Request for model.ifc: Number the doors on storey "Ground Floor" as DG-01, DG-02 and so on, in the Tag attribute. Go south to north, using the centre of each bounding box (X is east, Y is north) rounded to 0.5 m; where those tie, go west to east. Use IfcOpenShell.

First a look at what the model holds.

```python
import ifcopenshell
import ifcopenshell.util.element
import ifcopenshell.util.placement

model = ifcopenshell.open("model.ifc")
print(model.schema)
storey = next(s for s in model.by_type("IfcBuildingStorey") if s.Name == "Ground Floor")
doors = [e for e in ifcopenshell.util.element.get_decomposition(storey) if e.is_a("IfcDoor")]
for e in sorted(doors, key=lambda e: e.id()):
    origin = ifcopenshell.util.placement.get_local_placement(e.ObjectPlacement)[:3, 3]
    print(e.id(), e.Tag, e.Name, origin.round(2) + 0.0, sep=" | ")
```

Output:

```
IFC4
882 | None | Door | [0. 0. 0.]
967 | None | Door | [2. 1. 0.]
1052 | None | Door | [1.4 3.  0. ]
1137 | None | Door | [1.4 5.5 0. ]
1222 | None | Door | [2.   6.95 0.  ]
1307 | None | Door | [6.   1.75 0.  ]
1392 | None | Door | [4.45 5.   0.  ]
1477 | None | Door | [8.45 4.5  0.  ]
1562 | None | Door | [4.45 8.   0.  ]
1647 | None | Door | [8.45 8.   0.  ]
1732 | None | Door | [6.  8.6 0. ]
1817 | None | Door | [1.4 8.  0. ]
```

```python
import ifcopenshell
import ifcopenshell.geom
import ifcopenshell.util.element
import ifcopenshell.util.shape

model = ifcopenshell.open("model.ifc")
settings = ifcopenshell.geom.settings()
settings.set("use-world-coords", True)


def centre(element):
    shape = ifcopenshell.geom.create_shape(settings, element)
    return ifcopenshell.util.shape.get_bbox_centroid(shape.geometry)


storey = next(s for s in model.by_type("IfcBuildingStorey") if s.Name == "Ground Floor")
doors = [e for e in ifcopenshell.util.element.get_decomposition(storey) if e.is_a("IfcDoor")]

# Insertion points can sit at a corner or the storey origin, so sort by the geometry (in metres).
centres = {e: centre(e) for e in doors}
doors.sort(key=lambda e: (round(centres[e][1] / 0.5), centres[e][0]))

for i, e in enumerate(doors, start=1):
    number = f"DG-{i:02d}"
    e.Tag = number
    print(e.id(), number)

model.write("model_rev.ifc")
```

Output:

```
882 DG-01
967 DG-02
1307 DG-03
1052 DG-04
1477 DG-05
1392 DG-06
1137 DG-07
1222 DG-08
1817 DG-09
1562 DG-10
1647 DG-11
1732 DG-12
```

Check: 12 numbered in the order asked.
